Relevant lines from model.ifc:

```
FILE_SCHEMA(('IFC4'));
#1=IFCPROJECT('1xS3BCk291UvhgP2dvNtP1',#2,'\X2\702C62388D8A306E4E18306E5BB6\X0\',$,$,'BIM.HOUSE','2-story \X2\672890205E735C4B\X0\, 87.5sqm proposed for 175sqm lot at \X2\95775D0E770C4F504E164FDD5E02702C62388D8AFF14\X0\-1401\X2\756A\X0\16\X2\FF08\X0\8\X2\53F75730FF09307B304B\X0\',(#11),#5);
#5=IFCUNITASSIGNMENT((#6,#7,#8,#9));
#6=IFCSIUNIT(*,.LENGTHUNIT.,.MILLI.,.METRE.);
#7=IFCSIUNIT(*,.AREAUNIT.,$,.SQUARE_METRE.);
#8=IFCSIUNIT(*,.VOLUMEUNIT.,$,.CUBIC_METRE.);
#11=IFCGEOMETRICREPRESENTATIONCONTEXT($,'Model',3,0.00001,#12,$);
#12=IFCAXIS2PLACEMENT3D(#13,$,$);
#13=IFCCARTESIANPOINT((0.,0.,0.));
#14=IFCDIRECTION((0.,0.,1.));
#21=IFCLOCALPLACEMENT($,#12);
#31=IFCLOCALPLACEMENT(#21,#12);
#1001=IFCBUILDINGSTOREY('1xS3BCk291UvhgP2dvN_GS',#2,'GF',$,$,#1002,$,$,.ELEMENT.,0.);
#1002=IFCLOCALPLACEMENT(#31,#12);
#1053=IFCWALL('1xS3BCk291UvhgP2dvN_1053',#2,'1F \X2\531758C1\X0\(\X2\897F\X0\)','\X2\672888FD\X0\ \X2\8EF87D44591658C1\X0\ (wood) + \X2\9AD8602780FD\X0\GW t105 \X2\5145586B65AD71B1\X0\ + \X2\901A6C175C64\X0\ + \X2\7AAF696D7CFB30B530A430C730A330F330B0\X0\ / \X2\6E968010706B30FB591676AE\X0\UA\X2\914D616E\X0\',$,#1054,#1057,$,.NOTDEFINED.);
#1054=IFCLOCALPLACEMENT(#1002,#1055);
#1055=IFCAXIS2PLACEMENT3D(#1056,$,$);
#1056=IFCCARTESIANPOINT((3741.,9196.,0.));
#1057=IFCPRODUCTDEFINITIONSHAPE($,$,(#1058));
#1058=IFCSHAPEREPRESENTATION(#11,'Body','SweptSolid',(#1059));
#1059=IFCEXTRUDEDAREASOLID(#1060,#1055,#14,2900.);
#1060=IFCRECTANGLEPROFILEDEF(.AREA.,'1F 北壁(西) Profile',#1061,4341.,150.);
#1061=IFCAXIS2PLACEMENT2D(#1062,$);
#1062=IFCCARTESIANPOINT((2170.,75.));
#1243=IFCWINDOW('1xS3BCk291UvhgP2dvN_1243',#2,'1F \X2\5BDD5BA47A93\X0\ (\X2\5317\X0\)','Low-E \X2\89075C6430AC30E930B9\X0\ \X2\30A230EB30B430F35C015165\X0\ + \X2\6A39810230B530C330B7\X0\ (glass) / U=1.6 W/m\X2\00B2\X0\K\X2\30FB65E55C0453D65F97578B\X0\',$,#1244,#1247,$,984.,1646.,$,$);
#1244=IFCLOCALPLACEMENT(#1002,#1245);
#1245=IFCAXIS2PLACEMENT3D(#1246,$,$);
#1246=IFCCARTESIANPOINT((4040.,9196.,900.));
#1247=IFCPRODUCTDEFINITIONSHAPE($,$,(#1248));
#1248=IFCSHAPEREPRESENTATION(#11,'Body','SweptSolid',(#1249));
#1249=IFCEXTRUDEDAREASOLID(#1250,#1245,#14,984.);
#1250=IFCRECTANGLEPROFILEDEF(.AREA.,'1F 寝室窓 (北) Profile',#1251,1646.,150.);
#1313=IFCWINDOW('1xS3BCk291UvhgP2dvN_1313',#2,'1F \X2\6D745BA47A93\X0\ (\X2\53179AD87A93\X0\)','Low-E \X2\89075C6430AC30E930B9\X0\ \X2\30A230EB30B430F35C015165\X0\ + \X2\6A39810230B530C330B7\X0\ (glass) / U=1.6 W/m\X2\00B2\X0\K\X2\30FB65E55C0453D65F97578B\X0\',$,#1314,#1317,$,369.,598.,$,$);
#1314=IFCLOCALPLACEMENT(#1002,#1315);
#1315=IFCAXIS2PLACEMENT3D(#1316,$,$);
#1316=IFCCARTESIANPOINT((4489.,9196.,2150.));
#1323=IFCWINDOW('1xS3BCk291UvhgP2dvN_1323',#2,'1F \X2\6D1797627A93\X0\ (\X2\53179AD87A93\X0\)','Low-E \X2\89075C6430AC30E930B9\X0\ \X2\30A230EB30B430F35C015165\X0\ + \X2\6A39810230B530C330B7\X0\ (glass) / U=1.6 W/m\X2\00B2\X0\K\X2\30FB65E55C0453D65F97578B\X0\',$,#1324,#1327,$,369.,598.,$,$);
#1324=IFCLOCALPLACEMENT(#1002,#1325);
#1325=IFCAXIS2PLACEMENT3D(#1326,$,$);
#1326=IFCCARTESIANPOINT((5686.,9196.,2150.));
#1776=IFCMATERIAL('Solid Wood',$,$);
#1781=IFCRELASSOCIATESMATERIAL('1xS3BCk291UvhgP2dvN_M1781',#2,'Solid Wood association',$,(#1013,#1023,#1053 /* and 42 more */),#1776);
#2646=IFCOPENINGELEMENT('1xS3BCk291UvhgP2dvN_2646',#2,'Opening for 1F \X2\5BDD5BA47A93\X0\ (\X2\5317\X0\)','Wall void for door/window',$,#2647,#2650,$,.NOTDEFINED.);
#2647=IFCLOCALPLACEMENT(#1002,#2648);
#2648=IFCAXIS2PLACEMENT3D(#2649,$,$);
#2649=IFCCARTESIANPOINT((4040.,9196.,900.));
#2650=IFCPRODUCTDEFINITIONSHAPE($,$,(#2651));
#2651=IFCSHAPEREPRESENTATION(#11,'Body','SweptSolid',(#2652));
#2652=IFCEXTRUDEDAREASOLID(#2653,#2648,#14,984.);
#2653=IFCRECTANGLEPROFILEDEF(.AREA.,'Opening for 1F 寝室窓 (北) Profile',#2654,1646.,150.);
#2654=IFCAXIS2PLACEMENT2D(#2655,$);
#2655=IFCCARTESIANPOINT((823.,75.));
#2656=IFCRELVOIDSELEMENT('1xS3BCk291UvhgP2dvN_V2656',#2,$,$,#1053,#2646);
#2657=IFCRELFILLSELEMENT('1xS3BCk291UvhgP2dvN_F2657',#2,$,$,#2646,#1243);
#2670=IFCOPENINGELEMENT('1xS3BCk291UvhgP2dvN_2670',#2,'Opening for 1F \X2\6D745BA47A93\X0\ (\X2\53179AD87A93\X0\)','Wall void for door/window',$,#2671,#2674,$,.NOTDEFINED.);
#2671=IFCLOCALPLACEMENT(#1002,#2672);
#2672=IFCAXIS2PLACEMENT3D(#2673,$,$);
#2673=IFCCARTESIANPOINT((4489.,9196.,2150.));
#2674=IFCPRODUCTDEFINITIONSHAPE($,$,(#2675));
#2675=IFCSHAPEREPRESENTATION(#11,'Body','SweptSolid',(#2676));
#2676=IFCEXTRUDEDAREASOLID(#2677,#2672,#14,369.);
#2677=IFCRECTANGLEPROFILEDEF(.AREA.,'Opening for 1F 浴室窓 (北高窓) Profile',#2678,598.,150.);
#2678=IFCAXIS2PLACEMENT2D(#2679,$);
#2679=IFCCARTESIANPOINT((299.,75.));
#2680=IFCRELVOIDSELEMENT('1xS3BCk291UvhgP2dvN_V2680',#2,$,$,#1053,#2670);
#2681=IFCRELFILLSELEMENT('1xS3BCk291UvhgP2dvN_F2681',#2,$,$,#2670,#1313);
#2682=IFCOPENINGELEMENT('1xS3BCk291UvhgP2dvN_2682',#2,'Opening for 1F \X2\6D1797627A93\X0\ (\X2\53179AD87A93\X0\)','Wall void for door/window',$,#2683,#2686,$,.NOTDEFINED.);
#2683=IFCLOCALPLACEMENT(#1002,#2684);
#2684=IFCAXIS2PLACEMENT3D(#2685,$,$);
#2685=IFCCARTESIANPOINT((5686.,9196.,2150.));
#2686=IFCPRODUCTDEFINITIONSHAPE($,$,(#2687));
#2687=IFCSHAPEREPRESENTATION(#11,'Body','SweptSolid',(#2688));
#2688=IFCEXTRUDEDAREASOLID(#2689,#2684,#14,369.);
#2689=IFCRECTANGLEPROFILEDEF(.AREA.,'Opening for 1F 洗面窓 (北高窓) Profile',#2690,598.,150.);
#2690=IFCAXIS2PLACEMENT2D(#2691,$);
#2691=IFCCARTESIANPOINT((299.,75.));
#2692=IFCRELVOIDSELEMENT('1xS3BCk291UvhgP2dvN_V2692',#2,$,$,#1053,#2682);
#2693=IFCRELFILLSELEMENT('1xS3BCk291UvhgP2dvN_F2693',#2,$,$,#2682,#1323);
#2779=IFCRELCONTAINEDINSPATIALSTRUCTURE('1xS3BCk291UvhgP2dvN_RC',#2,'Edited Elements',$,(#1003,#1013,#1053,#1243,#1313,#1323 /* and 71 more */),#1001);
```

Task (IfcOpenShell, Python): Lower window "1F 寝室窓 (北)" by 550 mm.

```python
import numpy as np
import ifcopenshell
import ifcopenshell.api.geometry
import ifcopenshell.util.placement
import ifcopenshell.util.unit

model = ifcopenshell.open("model.ifc")
unit_scale = ifcopenshell.util.unit.calculate_unit_scale(model)

window = model.by_guid("1xS3BCk291UvhgP2dvN_1243")
opening = window.FillsVoids[0].RelatingOpeningElement
dz = -550.0

shift = np.array([0.0, 0.0, dz])
# The window is not placed relative to its opening, so move both.
for product in (opening, window):
    matrix = ifcopenshell.util.placement.get_local_placement(product.ObjectPlacement)
    matrix[:3, 3] += shift
    ifcopenshell.api.geometry.edit_object_placement(model, product=product, matrix=matrix, is_si=False)

print(f"moved by {dz * unit_scale:+.3f} m")

model.write("model_edited.ifc")
```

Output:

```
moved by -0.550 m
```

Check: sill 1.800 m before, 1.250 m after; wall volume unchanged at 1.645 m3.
